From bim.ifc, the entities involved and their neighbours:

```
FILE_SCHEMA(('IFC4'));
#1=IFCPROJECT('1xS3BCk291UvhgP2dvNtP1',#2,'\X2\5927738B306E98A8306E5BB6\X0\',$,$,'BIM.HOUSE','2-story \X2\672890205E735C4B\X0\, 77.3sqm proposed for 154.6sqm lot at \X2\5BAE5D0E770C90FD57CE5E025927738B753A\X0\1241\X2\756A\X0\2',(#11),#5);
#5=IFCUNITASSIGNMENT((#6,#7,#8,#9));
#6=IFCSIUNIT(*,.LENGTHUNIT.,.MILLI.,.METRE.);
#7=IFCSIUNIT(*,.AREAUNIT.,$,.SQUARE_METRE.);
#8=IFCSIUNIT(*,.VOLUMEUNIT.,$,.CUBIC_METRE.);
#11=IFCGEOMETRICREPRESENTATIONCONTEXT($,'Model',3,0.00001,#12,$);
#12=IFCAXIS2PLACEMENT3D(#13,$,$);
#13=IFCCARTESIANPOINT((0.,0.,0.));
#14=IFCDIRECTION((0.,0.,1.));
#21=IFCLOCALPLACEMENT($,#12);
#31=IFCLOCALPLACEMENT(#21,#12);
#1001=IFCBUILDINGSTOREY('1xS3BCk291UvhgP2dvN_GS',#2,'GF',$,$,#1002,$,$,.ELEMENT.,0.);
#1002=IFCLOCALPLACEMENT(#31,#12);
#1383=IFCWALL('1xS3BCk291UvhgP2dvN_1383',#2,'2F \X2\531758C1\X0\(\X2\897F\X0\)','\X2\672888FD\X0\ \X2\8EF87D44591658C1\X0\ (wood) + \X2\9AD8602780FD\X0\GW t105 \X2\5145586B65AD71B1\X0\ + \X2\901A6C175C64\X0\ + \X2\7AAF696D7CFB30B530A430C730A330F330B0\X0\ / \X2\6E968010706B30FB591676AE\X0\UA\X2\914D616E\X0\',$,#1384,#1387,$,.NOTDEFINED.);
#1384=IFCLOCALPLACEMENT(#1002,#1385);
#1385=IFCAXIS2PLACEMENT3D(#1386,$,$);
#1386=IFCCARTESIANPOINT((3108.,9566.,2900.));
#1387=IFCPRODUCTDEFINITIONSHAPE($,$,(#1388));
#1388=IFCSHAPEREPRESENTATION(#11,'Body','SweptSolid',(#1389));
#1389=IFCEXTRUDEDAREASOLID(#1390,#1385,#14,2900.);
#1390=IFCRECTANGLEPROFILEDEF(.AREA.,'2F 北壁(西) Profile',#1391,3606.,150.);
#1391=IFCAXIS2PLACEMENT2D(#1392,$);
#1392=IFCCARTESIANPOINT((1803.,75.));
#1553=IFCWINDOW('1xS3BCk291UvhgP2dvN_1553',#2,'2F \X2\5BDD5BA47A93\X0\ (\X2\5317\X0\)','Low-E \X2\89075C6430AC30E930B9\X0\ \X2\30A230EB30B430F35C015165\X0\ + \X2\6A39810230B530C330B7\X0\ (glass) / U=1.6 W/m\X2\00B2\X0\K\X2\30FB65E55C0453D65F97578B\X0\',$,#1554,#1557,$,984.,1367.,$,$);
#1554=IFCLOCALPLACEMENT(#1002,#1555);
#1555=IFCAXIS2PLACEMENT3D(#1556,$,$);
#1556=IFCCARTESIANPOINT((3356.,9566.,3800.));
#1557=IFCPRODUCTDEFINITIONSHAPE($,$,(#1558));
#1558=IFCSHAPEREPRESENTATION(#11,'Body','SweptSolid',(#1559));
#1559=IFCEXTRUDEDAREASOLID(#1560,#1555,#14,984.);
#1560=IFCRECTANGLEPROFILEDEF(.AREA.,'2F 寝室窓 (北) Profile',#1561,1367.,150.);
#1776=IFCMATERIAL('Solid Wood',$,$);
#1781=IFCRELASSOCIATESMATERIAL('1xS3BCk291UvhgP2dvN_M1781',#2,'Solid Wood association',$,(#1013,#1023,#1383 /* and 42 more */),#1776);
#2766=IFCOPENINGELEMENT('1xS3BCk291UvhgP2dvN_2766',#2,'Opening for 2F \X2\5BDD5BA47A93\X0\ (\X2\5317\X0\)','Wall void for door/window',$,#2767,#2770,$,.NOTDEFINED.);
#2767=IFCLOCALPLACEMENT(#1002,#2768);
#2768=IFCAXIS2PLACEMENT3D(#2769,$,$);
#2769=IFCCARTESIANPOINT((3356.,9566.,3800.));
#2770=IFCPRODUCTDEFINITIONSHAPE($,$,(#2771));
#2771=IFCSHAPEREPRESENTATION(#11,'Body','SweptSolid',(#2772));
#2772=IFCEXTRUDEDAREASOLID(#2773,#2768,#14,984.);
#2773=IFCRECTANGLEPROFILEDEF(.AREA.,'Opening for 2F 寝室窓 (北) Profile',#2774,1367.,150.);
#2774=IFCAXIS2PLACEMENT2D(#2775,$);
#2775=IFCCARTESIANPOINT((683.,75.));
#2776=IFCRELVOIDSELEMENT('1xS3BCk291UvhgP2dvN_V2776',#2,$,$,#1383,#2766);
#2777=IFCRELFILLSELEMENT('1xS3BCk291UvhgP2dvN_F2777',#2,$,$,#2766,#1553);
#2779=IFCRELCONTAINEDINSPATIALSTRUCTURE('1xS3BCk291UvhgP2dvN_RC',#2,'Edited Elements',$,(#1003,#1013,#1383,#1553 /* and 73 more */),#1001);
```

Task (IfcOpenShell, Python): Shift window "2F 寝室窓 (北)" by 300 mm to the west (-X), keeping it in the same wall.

```python
import ifcopenshell
import ifcopenshell.api.geometry
import ifcopenshell.util.placement
import ifcopenshell.util.unit

model = ifcopenshell.open("bim.ifc")
unit_scale = ifcopenshell.util.unit.calculate_unit_scale(model)

window = model.by_guid("1xS3BCk291UvhgP2dvN_1553")
opening = window.FillsVoids[0].RelatingOpeningElement
wall = opening.VoidsElements[0].RelatingBuildingElement

wall_matrix = ifcopenshell.util.placement.get_local_placement(wall.ObjectPlacement)
shift = wall_matrix[:3, 0] * -0.3 / unit_scale
before = ifcopenshell.util.placement.get_local_placement(window.ObjectPlacement)[:3, 3].copy()

# The window is not placed relative to its opening, so move both.
for product in (opening, window):
    matrix = ifcopenshell.util.placement.get_local_placement(product.ObjectPlacement)
    matrix[:3, 3] += shift
    ifcopenshell.api.geometry.edit_object_placement(model, product=product, matrix=matrix, is_si=False)

after = ifcopenshell.util.placement.get_local_placement(window.ObjectPlacement)[:3, 3]
print("window moved by", (after - before).round(3) + 0.0)

model.write("bim-out.ifc")
```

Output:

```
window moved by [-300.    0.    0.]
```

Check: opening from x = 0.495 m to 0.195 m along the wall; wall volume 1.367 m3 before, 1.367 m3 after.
